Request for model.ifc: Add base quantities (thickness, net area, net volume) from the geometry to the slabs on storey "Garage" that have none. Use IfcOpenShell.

First a look at what the model holds.

```python
import ifcopenshell
import ifcopenshell.util.element
import ifcopenshell.util.unit

model = ifcopenshell.open("model.ifc")
print(model.schema)
for unit_type in ("LENGTHUNIT", "AREAUNIT", "VOLUMEUNIT"):
    print(unit_type, ifcopenshell.util.unit.calculate_unit_scale(model, unit_type))
storey = next(s for s in model.by_type("IfcBuildingStorey") if s.Name == "Garage")
slabs = [e for e in ifcopenshell.util.element.get_decomposition(storey) if e.is_a("IfcSlab")]
for e in sorted(slabs, key=lambda e: e.id()):
    print(e.id(), e.is_a(), e.Name, list(ifcopenshell.util.element.get_psets(e, qtos_only=True)), sep=" | ")
```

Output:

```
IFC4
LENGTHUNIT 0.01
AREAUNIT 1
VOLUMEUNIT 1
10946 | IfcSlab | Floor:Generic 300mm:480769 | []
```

```python
import ifcopenshell
import ifcopenshell.api.pset
import ifcopenshell.geom
import ifcopenshell.util.element
import ifcopenshell.util.shape
import ifcopenshell.util.unit

model = ifcopenshell.open("model.ifc")
unit_scale = ifcopenshell.util.unit.calculate_unit_scale(model)
area_scale = ifcopenshell.util.unit.calculate_unit_scale(model, "AREAUNIT")
volume_scale = ifcopenshell.util.unit.calculate_unit_scale(model, "VOLUMEUNIT")
settings = ifcopenshell.geom.settings()

storey = next(s for s in model.by_type("IfcBuildingStorey") if s.Name == "Garage")
slabs = [e for e in ifcopenshell.util.element.get_decomposition(storey) if e.is_a("IfcSlab")]

for e in sorted(slabs, key=lambda e: e.id()):
    if ifcopenshell.util.element.get_psets(e, qtos_only=True, should_inherit=False):
        continue
    # Geometry comes back in metres, in the element's own axes.
    shape = ifcopenshell.geom.create_shape(settings, e)
    values = {
        "Width": ifcopenshell.util.shape.get_z(shape.geometry) / unit_scale,
        "NetArea": ifcopenshell.util.shape.get_footprint_area(shape.geometry) / area_scale,
        "NetVolume": ifcopenshell.util.shape.get_volume(shape.geometry) / volume_scale,
    }
    qto = ifcopenshell.api.pset.add_qto(model, product=e, name="Qto_SlabBaseQuantities")
    ifcopenshell.api.pset.edit_qto(model, qto=qto, properties=values)
    print(e.id(), {k: round(v, 3) for k, v in values.items()})

model.write("model-out.ifc")
```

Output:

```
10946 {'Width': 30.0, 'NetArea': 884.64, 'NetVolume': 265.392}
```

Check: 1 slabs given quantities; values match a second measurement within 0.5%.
